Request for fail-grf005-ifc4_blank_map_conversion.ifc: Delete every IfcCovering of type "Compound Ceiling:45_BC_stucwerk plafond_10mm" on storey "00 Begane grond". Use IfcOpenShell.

First a look at what the model holds.

```python
import ifcopenshell
import ifcopenshell.util.element

model = ifcopenshell.open("fail-grf005-ifc4_blank_map_conversion.ifc")
print(model.schema)
storey = next(s for s in model.by_type("IfcBuildingStorey") if s.Name == "00 Begane grond")
coverings = [e for e in ifcopenshell.util.element.get_decomposition(storey) if e.is_a("IfcCovering")]
seen = {}
for e in coverings:
    element_type = ifcopenshell.util.element.get_type(e)
    name = element_type.Name if element_type not in (None, e) else None
    seen[name] = seen.get(name, 0) + 1
for name, count in sorted(seen.items(), key=str):
    print(count, "x", name)
```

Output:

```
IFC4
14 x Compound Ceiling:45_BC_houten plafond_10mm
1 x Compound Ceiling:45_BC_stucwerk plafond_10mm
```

```python
import ifcopenshell
import ifcopenshell.api.root
import ifcopenshell.util.element

model = ifcopenshell.open("fail-grf005-ifc4_blank_map_conversion.ifc")

storey = next(s for s in model.by_type("IfcBuildingStorey") if s.Name == "00 Begane grond")
coverings = [e for e in ifcopenshell.util.element.get_decomposition(storey) if e.is_a("IfcCovering")]
targets = [e for e in coverings if (t := ifcopenshell.util.element.get_type(e)) not in (None, e) and t.Name == "Compound Ceiling:45_BC_stucwerk plafond_10mm"]

for e in targets:
    ifcopenshell.api.root.remove_product(model, product=e)
print(len(targets), "removed")

model.write("fail-grf005-ifc4_blank_map_conversion_edited.ifc")
```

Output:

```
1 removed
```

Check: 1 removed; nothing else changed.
